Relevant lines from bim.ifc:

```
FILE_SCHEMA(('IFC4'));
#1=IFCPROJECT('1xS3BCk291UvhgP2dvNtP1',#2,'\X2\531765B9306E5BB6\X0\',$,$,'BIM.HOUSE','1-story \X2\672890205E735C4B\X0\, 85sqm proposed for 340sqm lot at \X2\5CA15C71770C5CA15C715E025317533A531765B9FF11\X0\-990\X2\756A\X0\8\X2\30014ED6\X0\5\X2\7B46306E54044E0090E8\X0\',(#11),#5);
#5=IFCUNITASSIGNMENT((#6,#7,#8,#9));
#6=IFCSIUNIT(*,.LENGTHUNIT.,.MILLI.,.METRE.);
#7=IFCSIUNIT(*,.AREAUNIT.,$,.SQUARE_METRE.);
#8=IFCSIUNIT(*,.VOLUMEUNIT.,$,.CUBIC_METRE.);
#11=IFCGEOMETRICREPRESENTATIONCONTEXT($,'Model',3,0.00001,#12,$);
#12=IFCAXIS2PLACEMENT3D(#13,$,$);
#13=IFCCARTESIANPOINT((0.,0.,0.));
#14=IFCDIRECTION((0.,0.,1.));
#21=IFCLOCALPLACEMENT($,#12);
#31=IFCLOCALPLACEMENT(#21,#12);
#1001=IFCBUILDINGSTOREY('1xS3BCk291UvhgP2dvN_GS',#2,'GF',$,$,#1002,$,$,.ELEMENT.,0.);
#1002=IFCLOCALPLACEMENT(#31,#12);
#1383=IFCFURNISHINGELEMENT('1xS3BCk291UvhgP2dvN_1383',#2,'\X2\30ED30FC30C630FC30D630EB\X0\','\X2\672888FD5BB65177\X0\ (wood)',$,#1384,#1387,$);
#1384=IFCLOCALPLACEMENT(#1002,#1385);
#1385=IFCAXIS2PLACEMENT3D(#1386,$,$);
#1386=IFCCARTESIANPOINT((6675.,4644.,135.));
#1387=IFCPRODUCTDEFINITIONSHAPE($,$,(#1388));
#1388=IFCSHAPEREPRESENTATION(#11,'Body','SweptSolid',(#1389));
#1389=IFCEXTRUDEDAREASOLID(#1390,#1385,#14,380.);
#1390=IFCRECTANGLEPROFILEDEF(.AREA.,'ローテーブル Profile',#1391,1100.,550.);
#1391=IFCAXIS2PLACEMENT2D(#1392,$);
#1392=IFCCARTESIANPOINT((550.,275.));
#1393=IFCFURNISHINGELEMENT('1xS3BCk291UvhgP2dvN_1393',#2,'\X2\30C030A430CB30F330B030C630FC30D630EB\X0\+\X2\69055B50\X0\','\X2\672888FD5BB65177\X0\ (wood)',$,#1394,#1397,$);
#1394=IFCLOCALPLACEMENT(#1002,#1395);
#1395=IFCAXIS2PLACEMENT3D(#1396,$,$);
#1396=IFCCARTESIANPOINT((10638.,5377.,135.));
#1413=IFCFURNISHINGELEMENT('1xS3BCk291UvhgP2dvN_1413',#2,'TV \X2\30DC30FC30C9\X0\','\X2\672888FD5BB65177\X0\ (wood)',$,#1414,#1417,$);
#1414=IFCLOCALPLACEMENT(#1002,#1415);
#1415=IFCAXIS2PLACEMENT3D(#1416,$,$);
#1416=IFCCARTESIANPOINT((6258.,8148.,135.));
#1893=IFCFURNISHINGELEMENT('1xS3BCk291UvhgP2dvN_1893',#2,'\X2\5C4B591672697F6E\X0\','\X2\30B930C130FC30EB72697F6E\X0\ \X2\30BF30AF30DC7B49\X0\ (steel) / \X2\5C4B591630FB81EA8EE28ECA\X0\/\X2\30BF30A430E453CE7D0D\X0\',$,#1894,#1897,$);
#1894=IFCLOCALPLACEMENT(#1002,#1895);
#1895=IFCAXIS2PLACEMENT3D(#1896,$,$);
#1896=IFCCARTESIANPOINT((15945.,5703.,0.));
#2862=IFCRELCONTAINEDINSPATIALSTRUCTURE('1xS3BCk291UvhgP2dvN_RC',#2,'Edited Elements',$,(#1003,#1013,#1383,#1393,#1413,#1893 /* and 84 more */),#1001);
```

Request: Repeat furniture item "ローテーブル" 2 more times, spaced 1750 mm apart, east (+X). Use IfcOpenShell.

```python
import numpy as np
import ifcopenshell
import ifcopenshell.api.geometry
import ifcopenshell.api.root
import ifcopenshell.util.element
import ifcopenshell.util.placement

model = ifcopenshell.open("bim.ifc")


def reuse_history(source, copy):
    """copy_class also copies each property set's owner history, people and application; keep the originals."""
    for rel in copy.IsDefinedBy:
        if rel.is_a("IfcRelDefinesByProperties") and (history := rel.RelatingPropertyDefinition.OwnerHistory):
            rel.RelatingPropertyDefinition.OwnerHistory = source.OwnerHistory
            ifcopenshell.util.element.remove_deep2(model, history)


source = model.by_id(1383)
base = ifcopenshell.util.placement.get_local_placement(source.ObjectPlacement)
step = np.array([1.0, 0.0, 0.0]) * 1750.0

for i in range(1, 3):
    copy = ifcopenshell.api.root.copy_class(model, product=source)
    copy.Representation = ifcopenshell.util.element.copy_deep(
        model, source.Representation, exclude=["IfcGeometricRepresentationContext", "IfcRepresentationMap"]
    )
    reuse_history(source, copy)
    matrix = base.copy()
    matrix[:3, 3] += i * step
    print("added at", matrix[:3, 3].round(3) + 0.0)
    ifcopenshell.api.geometry.edit_object_placement(model, product=copy, matrix=matrix, is_si=False)

model.write("bim_edited.ifc")
```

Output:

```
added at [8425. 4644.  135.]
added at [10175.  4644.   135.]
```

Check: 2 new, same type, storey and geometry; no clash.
